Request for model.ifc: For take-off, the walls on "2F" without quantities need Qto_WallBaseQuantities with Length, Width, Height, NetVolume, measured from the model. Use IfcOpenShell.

First a look at what the model holds.

```python
import ifcopenshell
import ifcopenshell.util.element
import ifcopenshell.util.unit

model = ifcopenshell.open("model.ifc")
print(model.schema)
for unit_type in ("LENGTHUNIT", "AREAUNIT", "VOLUMEUNIT"):
    print(unit_type, ifcopenshell.util.unit.calculate_unit_scale(model, unit_type))
storey = next(s for s in model.by_type("IfcBuildingStorey") if s.Name == "2F")
walls = [e for e in ifcopenshell.util.element.get_decomposition(storey) if e.is_a("IfcWall")]
for e in sorted(walls, key=lambda e: e.id()):
    print(e.id(), e.is_a(), e.Name, list(ifcopenshell.util.element.get_psets(e, qtos_only=True)), sep=" | ")
```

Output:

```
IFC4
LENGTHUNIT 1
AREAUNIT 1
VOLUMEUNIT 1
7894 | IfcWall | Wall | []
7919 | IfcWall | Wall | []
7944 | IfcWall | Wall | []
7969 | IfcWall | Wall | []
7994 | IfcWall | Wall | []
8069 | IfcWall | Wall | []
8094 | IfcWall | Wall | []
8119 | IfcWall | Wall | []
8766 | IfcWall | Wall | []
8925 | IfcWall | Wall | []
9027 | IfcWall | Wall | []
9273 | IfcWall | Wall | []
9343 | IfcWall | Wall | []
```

```python
import ifcopenshell
import ifcopenshell.api.pset
import ifcopenshell.geom
import ifcopenshell.util.element
import ifcopenshell.util.shape
import ifcopenshell.util.unit

model = ifcopenshell.open("model.ifc")
unit_scale = ifcopenshell.util.unit.calculate_unit_scale(model)
volume_scale = ifcopenshell.util.unit.calculate_unit_scale(model, "VOLUMEUNIT")
settings = ifcopenshell.geom.settings()

storey = next(s for s in model.by_type("IfcBuildingStorey") if s.Name == "2F")
walls = [e for e in ifcopenshell.util.element.get_decomposition(storey) if e.is_a("IfcWall")]

for e in sorted(walls, key=lambda e: e.id()):
    if ifcopenshell.util.element.get_psets(e, qtos_only=True, should_inherit=False):
        continue
    # Geometry comes back in metres, in the element's own axes.
    shape = ifcopenshell.geom.create_shape(settings, e)
    values = {
        "Length": ifcopenshell.util.shape.get_x(shape.geometry) / unit_scale,
        "Width": ifcopenshell.util.shape.get_y(shape.geometry) / unit_scale,
        "Height": ifcopenshell.util.shape.get_z(shape.geometry) / unit_scale,
        "NetVolume": ifcopenshell.util.shape.get_volume(shape.geometry) / volume_scale,
    }
    qto = ifcopenshell.api.pset.add_qto(model, product=e, name="Qto_WallBaseQuantities")
    ifcopenshell.api.pset.edit_qto(model, qto=qto, properties=values)
    print(e.id(), {k: round(v, 3) for k, v in values.items()})

model.write("model_v2.ifc")
```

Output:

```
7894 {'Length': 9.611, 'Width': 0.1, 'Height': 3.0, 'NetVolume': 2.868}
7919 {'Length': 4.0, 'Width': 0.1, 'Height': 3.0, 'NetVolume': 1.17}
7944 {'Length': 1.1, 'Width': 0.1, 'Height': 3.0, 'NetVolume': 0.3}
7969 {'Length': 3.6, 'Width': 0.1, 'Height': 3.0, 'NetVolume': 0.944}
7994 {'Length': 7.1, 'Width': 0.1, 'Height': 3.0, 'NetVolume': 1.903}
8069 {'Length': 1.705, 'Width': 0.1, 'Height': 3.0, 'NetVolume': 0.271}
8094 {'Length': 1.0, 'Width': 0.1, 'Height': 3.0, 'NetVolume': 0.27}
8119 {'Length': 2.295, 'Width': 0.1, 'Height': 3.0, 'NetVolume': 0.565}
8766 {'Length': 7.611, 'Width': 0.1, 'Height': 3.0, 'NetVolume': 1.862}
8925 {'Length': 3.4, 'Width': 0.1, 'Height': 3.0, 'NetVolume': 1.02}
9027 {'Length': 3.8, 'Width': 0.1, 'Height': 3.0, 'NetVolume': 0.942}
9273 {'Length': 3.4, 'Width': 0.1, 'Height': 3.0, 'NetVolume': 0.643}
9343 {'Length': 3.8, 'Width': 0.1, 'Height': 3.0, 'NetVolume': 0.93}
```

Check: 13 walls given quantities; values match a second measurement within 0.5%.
